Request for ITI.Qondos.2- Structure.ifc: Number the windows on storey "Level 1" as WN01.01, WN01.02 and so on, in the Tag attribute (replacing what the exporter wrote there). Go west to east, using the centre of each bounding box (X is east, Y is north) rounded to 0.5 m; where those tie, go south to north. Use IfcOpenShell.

First a look at what the model holds.

```python
import ifcopenshell
import ifcopenshell.util.element
import ifcopenshell.util.placement

model = ifcopenshell.open("ITI.Qondos.2- Structure.ifc")
print(model.schema)
storey = next(s for s in model.by_type("IfcBuildingStorey") if s.Name == "Level 1")
windows = [e for e in ifcopenshell.util.element.get_decomposition(storey) if e.is_a("IfcWindow")]
for e in sorted(windows, key=lambda e: e.id()):
    origin = ifcopenshell.util.placement.get_local_placement(e.ObjectPlacement)[:3, 3]
    print(e.id(), e.Tag, e.Name, origin.round(2) + 0.0, sep=" | ")
```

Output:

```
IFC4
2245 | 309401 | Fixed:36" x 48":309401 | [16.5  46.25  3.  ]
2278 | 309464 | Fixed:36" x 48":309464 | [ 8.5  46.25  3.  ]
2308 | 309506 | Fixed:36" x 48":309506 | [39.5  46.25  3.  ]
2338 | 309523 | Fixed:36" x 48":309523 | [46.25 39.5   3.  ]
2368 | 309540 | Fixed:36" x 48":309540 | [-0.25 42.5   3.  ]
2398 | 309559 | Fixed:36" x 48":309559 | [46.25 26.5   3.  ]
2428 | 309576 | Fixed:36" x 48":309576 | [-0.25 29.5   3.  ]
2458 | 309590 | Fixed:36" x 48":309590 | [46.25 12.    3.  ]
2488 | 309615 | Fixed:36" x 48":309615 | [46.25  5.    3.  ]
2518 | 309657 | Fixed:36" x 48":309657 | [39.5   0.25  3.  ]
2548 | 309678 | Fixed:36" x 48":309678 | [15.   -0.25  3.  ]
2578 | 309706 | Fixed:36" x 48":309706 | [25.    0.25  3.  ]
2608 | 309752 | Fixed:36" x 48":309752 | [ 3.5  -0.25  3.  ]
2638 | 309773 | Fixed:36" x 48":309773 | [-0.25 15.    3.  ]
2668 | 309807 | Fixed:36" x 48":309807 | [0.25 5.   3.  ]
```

```python
import ifcopenshell
import ifcopenshell.geom
import ifcopenshell.util.element
import ifcopenshell.util.shape

model = ifcopenshell.open("ITI.Qondos.2- Structure.ifc")
settings = ifcopenshell.geom.settings()
settings.set("use-world-coords", True)


def centre(element):
    shape = ifcopenshell.geom.create_shape(settings, element)
    return ifcopenshell.util.shape.get_bbox_centroid(shape.geometry)


storey = next(s for s in model.by_type("IfcBuildingStorey") if s.Name == "Level 1")
windows = [e for e in ifcopenshell.util.element.get_decomposition(storey) if e.is_a("IfcWindow")]

# Insertion points can sit at a corner or the storey origin, so sort by the geometry (in metres).
centres = {e: centre(e) for e in windows}
windows.sort(key=lambda e: (round(centres[e][0] / 0.5), centres[e][1]))

for i, e in enumerate(windows, start=1):
    number = f"WN01.{i:02d}"
    e.Tag = number
    print(e.id(), number)

model.write("ITI.Qondos.2- Structure_edited.ifc")
```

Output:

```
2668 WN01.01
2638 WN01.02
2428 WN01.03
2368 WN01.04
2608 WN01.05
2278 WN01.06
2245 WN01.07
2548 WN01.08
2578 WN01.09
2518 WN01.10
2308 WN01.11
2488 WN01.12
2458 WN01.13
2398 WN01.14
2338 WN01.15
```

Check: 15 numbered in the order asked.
